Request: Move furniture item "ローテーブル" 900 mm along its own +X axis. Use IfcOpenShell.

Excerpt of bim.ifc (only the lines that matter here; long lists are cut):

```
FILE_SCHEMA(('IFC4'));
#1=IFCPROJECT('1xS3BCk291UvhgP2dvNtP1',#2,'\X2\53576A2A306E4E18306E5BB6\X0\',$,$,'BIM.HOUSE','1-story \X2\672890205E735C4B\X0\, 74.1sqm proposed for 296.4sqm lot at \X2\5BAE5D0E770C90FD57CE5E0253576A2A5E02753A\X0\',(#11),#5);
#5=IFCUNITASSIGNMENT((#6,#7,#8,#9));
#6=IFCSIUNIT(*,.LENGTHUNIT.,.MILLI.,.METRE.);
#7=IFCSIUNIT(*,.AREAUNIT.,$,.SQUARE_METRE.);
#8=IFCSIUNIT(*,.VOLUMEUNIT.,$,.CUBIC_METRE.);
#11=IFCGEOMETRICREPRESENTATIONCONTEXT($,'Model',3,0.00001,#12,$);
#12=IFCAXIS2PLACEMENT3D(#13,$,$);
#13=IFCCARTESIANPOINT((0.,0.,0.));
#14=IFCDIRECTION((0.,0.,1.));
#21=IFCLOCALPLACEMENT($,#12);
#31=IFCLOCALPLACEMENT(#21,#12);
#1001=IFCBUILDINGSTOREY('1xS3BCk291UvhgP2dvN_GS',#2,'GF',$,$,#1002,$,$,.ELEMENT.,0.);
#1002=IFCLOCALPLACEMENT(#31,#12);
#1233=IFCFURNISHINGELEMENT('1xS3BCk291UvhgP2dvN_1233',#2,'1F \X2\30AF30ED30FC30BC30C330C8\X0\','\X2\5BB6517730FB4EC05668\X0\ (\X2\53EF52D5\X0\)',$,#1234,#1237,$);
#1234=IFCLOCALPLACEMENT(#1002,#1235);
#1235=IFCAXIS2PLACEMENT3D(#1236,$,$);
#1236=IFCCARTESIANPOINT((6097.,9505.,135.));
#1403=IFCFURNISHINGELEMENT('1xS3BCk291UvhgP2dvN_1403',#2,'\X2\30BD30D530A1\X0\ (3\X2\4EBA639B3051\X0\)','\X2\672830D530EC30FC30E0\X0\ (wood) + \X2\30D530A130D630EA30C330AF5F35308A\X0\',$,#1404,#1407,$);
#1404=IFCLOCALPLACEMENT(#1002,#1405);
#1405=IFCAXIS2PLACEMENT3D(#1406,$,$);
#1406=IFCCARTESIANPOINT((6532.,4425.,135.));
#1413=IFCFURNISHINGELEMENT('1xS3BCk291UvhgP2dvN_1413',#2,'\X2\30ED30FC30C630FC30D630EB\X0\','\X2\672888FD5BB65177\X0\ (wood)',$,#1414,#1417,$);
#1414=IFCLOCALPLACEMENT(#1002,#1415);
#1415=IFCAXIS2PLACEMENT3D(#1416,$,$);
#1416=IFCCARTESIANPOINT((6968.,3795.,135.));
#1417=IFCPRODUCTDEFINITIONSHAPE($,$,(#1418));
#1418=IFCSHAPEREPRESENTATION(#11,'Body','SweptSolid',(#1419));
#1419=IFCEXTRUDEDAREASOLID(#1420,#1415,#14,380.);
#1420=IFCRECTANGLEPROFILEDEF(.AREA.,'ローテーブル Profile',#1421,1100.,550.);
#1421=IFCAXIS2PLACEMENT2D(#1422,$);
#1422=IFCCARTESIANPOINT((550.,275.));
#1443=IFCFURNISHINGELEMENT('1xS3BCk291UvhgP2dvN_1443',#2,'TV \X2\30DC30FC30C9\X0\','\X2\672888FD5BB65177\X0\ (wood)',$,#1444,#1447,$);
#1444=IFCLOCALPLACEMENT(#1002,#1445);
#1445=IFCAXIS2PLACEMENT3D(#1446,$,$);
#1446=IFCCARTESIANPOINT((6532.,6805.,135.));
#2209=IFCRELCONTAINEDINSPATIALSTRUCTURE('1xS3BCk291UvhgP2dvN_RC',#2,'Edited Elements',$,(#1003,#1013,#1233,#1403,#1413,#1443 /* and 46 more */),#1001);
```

```python
import ifcopenshell
import ifcopenshell.api.geometry
import ifcopenshell.util.placement
import ifcopenshell.util.unit

model = ifcopenshell.open("bim.ifc")
unit_scale = ifcopenshell.util.unit.calculate_unit_scale(model)

item = model.by_guid("1xS3BCk291UvhgP2dvN_1413")
matrix = ifcopenshell.util.placement.get_local_placement(item.ObjectPlacement)
matrix[:3, 3] += matrix[:3, 0] * 0.9 / unit_scale
ifcopenshell.api.geometry.edit_object_placement(model, product=item, matrix=matrix, is_si=False)

print(ifcopenshell.util.placement.get_local_placement(item.ObjectPlacement).round(3) + 0.0)

model.write("bim_edited.ifc")
```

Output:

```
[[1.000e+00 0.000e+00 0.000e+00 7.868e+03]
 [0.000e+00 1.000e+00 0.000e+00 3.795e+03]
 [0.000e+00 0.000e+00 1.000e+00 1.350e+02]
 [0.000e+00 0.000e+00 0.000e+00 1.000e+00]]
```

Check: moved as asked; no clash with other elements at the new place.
